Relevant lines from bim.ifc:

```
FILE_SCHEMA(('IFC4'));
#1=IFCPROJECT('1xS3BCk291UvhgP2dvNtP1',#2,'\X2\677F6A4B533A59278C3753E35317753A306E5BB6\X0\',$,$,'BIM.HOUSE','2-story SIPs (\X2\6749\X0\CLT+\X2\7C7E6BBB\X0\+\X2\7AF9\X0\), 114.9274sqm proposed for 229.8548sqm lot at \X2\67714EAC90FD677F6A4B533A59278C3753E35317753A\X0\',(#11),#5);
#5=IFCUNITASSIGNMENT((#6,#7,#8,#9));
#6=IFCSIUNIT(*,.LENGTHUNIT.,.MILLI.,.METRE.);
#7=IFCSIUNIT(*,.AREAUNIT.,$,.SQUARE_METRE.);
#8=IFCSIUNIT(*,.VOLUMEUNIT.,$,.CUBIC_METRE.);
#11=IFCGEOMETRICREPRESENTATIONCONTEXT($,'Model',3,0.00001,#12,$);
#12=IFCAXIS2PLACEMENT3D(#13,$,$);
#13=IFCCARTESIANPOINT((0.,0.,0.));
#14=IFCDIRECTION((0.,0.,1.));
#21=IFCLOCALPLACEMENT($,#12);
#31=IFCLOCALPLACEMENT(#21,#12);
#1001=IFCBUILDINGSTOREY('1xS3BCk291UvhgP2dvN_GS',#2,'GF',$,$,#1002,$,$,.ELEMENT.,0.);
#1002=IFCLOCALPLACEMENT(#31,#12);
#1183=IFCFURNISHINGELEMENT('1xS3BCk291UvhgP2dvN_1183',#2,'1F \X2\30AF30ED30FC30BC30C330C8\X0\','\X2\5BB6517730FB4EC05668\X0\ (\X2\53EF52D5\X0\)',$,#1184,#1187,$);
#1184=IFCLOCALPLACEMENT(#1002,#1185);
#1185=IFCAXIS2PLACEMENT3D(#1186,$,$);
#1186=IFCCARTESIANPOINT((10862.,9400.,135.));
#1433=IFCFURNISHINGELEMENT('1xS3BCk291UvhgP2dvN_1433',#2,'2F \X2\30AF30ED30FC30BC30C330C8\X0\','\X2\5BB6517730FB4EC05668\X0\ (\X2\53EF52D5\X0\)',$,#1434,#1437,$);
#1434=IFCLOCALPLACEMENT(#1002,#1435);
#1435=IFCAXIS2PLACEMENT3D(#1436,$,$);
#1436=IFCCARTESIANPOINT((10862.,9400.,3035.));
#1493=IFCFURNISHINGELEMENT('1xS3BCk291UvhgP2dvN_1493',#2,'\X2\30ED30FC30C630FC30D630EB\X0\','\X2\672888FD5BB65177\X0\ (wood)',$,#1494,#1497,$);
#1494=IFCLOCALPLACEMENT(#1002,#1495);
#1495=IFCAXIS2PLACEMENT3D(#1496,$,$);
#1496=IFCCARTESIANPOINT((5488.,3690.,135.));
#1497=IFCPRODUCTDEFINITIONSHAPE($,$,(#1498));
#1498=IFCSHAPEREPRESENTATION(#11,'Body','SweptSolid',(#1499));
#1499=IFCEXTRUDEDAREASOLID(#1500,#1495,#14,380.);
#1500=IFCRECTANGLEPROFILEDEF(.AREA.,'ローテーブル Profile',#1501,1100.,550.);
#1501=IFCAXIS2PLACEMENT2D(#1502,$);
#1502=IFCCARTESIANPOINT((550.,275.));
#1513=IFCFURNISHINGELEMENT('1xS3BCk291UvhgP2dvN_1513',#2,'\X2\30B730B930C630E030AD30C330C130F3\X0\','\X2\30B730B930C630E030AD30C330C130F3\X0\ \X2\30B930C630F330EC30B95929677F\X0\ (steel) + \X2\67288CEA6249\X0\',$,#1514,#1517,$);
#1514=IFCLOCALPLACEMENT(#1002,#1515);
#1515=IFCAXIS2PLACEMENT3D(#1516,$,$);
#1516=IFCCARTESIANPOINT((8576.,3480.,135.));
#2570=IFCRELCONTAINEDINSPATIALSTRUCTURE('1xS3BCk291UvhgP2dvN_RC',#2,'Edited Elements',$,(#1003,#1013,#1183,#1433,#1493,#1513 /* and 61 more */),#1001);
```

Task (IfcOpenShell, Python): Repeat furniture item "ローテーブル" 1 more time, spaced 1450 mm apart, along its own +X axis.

```python
import ifcopenshell
import ifcopenshell.api.geometry
import ifcopenshell.api.root
import ifcopenshell.util.element
import ifcopenshell.util.placement
import ifcopenshell.util.unit

model = ifcopenshell.open("bim.ifc")
unit_scale = ifcopenshell.util.unit.calculate_unit_scale(model)


def reuse_history(source, copy):
    """copy_class also copies each property set's owner history, people and application; keep the originals."""
    for rel in copy.IsDefinedBy:
        if rel.is_a("IfcRelDefinesByProperties") and (history := rel.RelatingPropertyDefinition.OwnerHistory):
            rel.RelatingPropertyDefinition.OwnerHistory = source.OwnerHistory
            ifcopenshell.util.element.remove_deep2(model, history)


source = model.by_id(1493)
base = ifcopenshell.util.placement.get_local_placement(source.ObjectPlacement)
step = base[:3, 0] * 1.45 / unit_scale

for i in range(1, 2):
    copy = ifcopenshell.api.root.copy_class(model, product=source)
    copy.Representation = ifcopenshell.util.element.copy_deep(
        model, source.Representation, exclude=["IfcGeometricRepresentationContext", "IfcRepresentationMap"]
    )
    reuse_history(source, copy)
    matrix = base.copy()
    matrix[:3, 3] += i * step
    print("added at", matrix[:3, 3].round(3) + 0.0)
    ifcopenshell.api.geometry.edit_object_placement(model, product=copy, matrix=matrix, is_si=False)

model.write("bim-out.ifc")
```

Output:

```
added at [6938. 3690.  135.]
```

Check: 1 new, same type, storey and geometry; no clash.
